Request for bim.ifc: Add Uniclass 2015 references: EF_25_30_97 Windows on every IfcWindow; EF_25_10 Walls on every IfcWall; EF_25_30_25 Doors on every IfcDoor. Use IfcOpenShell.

First a look at what the model holds.

```python
import ifcopenshell

model = ifcopenshell.open("bim.ifc")
print(model.schema)
print("classifications:", [c.Name for c in model.by_type("IfcClassification")])
for ifc_class in ("IfcDoor", "IfcRoof", "IfcStair", "IfcWall", "IfcWindow"):
    print(ifc_class, len(model.by_type(ifc_class)))
```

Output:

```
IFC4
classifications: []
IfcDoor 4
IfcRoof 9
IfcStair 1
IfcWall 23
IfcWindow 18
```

```python
import ifcopenshell
import ifcopenshell.api.classification

model = ifcopenshell.open("bim.ifc")

system = ifcopenshell.api.classification.add_classification(model, classification="Uniclass 2015")

codes = {
    "IfcWindow": ("EF_25_30_97", "Windows"),
    "IfcWall": ("EF_25_10", "Walls"),
    "IfcDoor": ("EF_25_30_25", "Doors"),
}
for ifc_class, (code, name) in codes.items():
    products = model.by_type(ifc_class)
    ifcopenshell.api.classification.add_reference(
        model, products=products, classification=system, identification=code, name=name
    )
    print(code, len(products))

model.write("bim_rev.ifc")
```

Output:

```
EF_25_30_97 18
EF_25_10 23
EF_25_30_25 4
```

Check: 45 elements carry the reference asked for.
